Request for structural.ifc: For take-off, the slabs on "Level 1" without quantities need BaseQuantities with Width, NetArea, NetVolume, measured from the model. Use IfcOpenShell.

First a look at what the model holds.

```python
import ifcopenshell
import ifcopenshell.util.element
import ifcopenshell.util.unit

model = ifcopenshell.open("structural.ifc")
print(model.schema)
for unit_type in ("LENGTHUNIT", "AREAUNIT", "VOLUMEUNIT"):
    print(unit_type, ifcopenshell.util.unit.calculate_unit_scale(model, unit_type))
storey = next(s for s in model.by_type("IfcBuildingStorey") if s.Name == "Level 1")
slabs = [e for e in ifcopenshell.util.element.get_decomposition(storey) if e.is_a("IfcSlab")]
for e in sorted(slabs, key=lambda e: e.id()):
    print(e.id(), e.is_a(), e.Name, list(ifcopenshell.util.element.get_psets(e, qtos_only=True)), sep=" | ")
```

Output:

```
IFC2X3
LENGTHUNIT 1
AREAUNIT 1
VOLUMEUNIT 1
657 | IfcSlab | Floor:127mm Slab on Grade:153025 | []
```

```python
import ifcopenshell
import ifcopenshell.api.pset
import ifcopenshell.geom
import ifcopenshell.util.element
import ifcopenshell.util.shape
import ifcopenshell.util.unit

model = ifcopenshell.open("structural.ifc")
unit_scale = ifcopenshell.util.unit.calculate_unit_scale(model)
area_scale = ifcopenshell.util.unit.calculate_unit_scale(model, "AREAUNIT")
volume_scale = ifcopenshell.util.unit.calculate_unit_scale(model, "VOLUMEUNIT")
settings = ifcopenshell.geom.settings()

storey = next(s for s in model.by_type("IfcBuildingStorey") if s.Name == "Level 1")
slabs = [e for e in ifcopenshell.util.element.get_decomposition(storey) if e.is_a("IfcSlab")]

for e in sorted(slabs, key=lambda e: e.id()):
    if ifcopenshell.util.element.get_psets(e, qtos_only=True, should_inherit=False):
        continue
    # Geometry comes back in metres, in the element's own axes.
    shape = ifcopenshell.geom.create_shape(settings, e)
    values = {
        "Width": ifcopenshell.util.shape.get_z(shape.geometry) / unit_scale,
        "NetArea": ifcopenshell.util.shape.get_footprint_area(shape.geometry) / area_scale,
        "NetVolume": ifcopenshell.util.shape.get_volume(shape.geometry) / volume_scale,
    }
    qto = ifcopenshell.api.pset.add_qto(model, product=e, name="BaseQuantities")
    ifcopenshell.api.pset.edit_qto(model, qto=qto, properties=values)
    print(e.id(), {k: round(v, 3) for k, v in values.items()})

model.write("structural_updated.ifc")
```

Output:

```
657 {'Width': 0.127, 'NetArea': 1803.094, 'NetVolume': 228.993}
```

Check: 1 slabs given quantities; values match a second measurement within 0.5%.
